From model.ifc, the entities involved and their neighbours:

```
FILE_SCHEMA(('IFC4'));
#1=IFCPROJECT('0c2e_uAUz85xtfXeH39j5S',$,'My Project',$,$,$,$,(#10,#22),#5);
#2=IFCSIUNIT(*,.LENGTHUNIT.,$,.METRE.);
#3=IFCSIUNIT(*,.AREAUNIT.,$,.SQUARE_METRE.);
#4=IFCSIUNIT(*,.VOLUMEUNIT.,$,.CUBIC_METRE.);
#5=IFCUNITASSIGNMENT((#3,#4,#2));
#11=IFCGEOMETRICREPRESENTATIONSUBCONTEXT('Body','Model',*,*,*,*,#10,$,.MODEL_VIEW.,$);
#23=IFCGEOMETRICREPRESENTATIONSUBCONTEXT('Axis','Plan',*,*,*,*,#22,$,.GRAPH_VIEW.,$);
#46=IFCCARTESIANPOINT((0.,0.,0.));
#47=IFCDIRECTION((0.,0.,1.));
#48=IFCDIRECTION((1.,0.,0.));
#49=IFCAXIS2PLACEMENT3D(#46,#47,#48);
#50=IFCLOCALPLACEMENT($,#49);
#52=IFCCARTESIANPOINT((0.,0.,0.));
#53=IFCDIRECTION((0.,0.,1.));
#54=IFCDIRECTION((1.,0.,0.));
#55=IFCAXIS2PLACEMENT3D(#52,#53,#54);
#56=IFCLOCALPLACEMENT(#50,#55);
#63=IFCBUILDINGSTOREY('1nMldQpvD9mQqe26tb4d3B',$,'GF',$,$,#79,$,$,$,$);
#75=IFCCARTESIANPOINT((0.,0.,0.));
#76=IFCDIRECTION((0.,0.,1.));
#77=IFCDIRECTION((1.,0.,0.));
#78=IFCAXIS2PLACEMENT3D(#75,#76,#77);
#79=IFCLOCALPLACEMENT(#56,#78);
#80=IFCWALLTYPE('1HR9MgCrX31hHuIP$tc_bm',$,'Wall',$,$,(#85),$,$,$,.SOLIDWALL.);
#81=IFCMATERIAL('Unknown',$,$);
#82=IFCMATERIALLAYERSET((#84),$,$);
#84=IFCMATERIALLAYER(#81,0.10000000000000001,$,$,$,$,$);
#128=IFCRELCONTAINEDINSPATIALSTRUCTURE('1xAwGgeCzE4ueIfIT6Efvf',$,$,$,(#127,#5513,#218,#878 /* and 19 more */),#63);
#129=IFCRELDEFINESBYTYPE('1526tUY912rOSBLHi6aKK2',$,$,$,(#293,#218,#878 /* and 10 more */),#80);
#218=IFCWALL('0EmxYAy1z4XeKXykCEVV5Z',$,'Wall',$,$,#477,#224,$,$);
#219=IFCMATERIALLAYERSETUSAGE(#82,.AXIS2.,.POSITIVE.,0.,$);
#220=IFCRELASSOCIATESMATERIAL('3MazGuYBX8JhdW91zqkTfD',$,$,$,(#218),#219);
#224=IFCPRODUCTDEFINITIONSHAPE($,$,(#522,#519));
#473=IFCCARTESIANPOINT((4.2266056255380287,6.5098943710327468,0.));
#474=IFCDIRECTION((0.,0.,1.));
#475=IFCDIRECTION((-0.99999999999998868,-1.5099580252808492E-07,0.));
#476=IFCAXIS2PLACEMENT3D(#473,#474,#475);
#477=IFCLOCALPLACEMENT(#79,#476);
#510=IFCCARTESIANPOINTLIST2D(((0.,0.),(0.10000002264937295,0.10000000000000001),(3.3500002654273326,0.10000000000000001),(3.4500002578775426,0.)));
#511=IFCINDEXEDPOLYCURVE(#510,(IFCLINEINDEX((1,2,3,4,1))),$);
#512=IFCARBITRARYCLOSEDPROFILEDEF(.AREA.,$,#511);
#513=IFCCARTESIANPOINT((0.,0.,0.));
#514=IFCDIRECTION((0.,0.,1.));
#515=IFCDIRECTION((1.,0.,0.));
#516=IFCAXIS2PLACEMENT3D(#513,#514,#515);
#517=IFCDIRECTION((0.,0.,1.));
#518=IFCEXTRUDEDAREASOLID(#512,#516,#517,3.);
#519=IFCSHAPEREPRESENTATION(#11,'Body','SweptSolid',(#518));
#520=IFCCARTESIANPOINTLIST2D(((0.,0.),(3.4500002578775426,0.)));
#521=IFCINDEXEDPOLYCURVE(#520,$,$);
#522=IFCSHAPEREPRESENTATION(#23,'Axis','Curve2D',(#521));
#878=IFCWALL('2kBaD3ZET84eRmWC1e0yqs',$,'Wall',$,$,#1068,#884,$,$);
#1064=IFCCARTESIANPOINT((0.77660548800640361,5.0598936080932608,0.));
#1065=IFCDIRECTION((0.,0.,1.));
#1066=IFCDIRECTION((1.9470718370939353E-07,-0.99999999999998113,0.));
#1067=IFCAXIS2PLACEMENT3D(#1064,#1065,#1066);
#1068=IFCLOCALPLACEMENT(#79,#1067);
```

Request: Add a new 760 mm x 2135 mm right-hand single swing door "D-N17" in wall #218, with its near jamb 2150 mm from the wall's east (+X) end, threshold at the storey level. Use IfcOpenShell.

```python
import numpy as np
import ifcopenshell
import ifcopenshell.api.feature
import ifcopenshell.api.geometry
import ifcopenshell.api.root
import ifcopenshell.api.spatial
import ifcopenshell.geom
import ifcopenshell.util.element
import ifcopenshell.util.placement
import ifcopenshell.util.representation
import ifcopenshell.util.shape
import ifcopenshell.util.unit

model = ifcopenshell.open("model.ifc")
unit_scale = ifcopenshell.util.unit.calculate_unit_scale(model)
settings = ifcopenshell.geom.settings()


def volume(element):
    """Net volume in cubic metres, openings subtracted."""
    shape = ifcopenshell.geom.create_shape(settings, element)
    return ifcopenshell.util.shape.get_volume(shape.geometry)


wall = model.by_guid("0EmxYAy1z4XeKXykCEVV5Z")
storey = ifcopenshell.util.element.get_container(wall, ifc_class="IfcBuildingStorey")
context = ifcopenshell.util.representation.get_context(model, "Model", "Body", "MODEL_VIEW")
before = volume(wall)

width, height, from_end, sill = 0.76, 2.135, 2.15, 0.0  # metres

# The wall runs along its own X axis, and the end named is its -X end.
wall_shape = ifcopenshell.geom.create_shape(settings, wall)
x, y, z = ifcopenshell.util.shape.get_vertices(wall_shape.geometry).T
start = x.min() + from_end
face, thickness = float(y.min()), float(y.max() - y.min())
wall_matrix = ifcopenshell.util.placement.get_local_placement(wall.ObjectPlacement)
level = ifcopenshell.util.placement.get_local_placement(storey.ObjectPlacement)[2, 3]


def in_wall(x, y):
    """Placement at x, y metres in the wall's axes, at sill height."""
    matrix = wall_matrix.copy()
    matrix[:, 3] = wall_matrix @ np.array([x / unit_scale, y / unit_scale, 0.0, 1.0])
    matrix[2, 3] = level + sill / unit_scale
    return matrix


# Opening: a box that overshoots both wall faces by 50 mm.
opening = ifcopenshell.api.root.create_entity(model, ifc_class="IfcOpeningElement", predefined_type="OPENING")
box = ifcopenshell.api.geometry.add_wall_representation(
    model, context=context, length=width, height=height, thickness=thickness + 0.1
)
ifcopenshell.api.geometry.assign_representation(model, product=opening, representation=box)
ifcopenshell.api.geometry.edit_object_placement(model, product=opening, matrix=in_wall(start, face - 0.05), is_si=False)
ifcopenshell.api.feature.add_feature(model, feature=opening, element=wall)

door = ifcopenshell.api.root.create_entity(model, ifc_class="IfcDoor", name="D-N17", predefined_type="DOOR")
door.OverallWidth, door.OverallHeight = width / unit_scale, height / unit_scale
door.OperationType = "SINGLE_SWING_RIGHT"
body = ifcopenshell.api.geometry.add_door_representation(
    model,
    context=context,
    overall_width=door.OverallWidth,
    overall_height=door.OverallHeight,
    operation_type="SINGLE_SWING_RIGHT",
    lining_properties={"LiningDepth": thickness / unit_scale, "ThresholdDepth": thickness / unit_scale},
)
ifcopenshell.api.geometry.assign_representation(model, product=door, representation=body)
ifcopenshell.api.spatial.assign_container(model, products=[door], relating_structure=storey)
ifcopenshell.api.feature.add_filling(model, opening=opening, element=door)

# The lining spans the wall, so the door starts at the wall face.
ifcopenshell.api.geometry.edit_object_placement(model, product=door, matrix=in_wall(start, face), is_si=False)

after = volume(wall)

print(f"wall volume {before:.3f} -> {after:.3f} m3")

model.write("model_v2.ifc")
```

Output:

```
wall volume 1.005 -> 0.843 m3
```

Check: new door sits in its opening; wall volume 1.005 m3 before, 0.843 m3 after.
